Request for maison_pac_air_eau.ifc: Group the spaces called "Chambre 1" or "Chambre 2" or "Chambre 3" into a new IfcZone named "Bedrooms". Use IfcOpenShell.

First a look at what the model holds.

```python
import ifcopenshell

model = ifcopenshell.open("maison_pac_air_eau.ifc")
print(model.schema)
seen = {}
for space in model.by_type("IfcSpace"):
    seen[space.LongName] = seen.get(space.LongName, 0) + 1
for name, count in sorted(seen.items(), key=str):
    print(count, "x", name)
print("zones:", [z.Name for z in model.by_type("IfcZone")][:20])
```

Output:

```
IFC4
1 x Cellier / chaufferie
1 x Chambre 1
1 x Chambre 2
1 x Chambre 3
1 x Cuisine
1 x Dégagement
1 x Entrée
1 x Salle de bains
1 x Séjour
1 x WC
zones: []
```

```python
import ifcopenshell
import ifcopenshell.api.group
import ifcopenshell.api.root

model = ifcopenshell.open("maison_pac_air_eau.ifc")

names = {"Chambre 1", "Chambre 2", "Chambre 3"}
spaces = [s for s in model.by_type("IfcSpace") if s.LongName in names]

zone = ifcopenshell.api.root.create_entity(model, ifc_class="IfcZone", name="Bedrooms")
ifcopenshell.api.group.assign_group(model, products=spaces, group=zone)
print(len(spaces), "spaces in", zone.Name)

model.write("maison_pac_air_eau_rev.ifc")
```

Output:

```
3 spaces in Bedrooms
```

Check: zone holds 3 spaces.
